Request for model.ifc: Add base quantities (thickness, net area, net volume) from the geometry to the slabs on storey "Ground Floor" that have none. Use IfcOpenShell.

First a look at what the model holds.

```python
import ifcopenshell
import ifcopenshell.util.element
import ifcopenshell.util.unit

model = ifcopenshell.open("model.ifc")
print(model.schema)
for unit_type in ("LENGTHUNIT", "AREAUNIT", "VOLUMEUNIT"):
    print(unit_type, ifcopenshell.util.unit.calculate_unit_scale(model, unit_type))
storey = next(s for s in model.by_type("IfcBuildingStorey") if s.Name == "Ground Floor")
slabs = [e for e in ifcopenshell.util.element.get_decomposition(storey) if e.is_a("IfcSlab")]
for e in sorted(slabs, key=lambda e: e.id()):
    print(e.id(), e.is_a(), e.Name, list(ifcopenshell.util.element.get_psets(e, qtos_only=True)), sep=" | ")
```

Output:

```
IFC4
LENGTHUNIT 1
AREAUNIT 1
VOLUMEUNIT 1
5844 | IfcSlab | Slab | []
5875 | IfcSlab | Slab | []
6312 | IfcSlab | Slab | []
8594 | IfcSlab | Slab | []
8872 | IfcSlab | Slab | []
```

```python
import ifcopenshell
import ifcopenshell.api.pset
import ifcopenshell.geom
import ifcopenshell.util.element
import ifcopenshell.util.shape
import ifcopenshell.util.unit

model = ifcopenshell.open("model.ifc")
unit_scale = ifcopenshell.util.unit.calculate_unit_scale(model)
area_scale = ifcopenshell.util.unit.calculate_unit_scale(model, "AREAUNIT")
volume_scale = ifcopenshell.util.unit.calculate_unit_scale(model, "VOLUMEUNIT")
settings = ifcopenshell.geom.settings()

storey = next(s for s in model.by_type("IfcBuildingStorey") if s.Name == "Ground Floor")
slabs = [e for e in ifcopenshell.util.element.get_decomposition(storey) if e.is_a("IfcSlab")]

for e in sorted(slabs, key=lambda e: e.id()):
    if ifcopenshell.util.element.get_psets(e, qtos_only=True, should_inherit=False):
        continue
    # Geometry comes back in metres, in the element's own axes.
    shape = ifcopenshell.geom.create_shape(settings, e)
    values = {
        "Width": ifcopenshell.util.shape.get_z(shape.geometry) / unit_scale,
        "NetArea": ifcopenshell.util.shape.get_footprint_area(shape.geometry) / area_scale,
        "NetVolume": ifcopenshell.util.shape.get_volume(shape.geometry) / volume_scale,
    }
    qto = ifcopenshell.api.pset.add_qto(model, product=e, name="Qto_SlabBaseQuantities")
    ifcopenshell.api.pset.edit_qto(model, qto=qto, properties=values)
    print(e.id(), {k: round(v, 3) for k, v in values.items()})

model.write("model_updated.ifc")
```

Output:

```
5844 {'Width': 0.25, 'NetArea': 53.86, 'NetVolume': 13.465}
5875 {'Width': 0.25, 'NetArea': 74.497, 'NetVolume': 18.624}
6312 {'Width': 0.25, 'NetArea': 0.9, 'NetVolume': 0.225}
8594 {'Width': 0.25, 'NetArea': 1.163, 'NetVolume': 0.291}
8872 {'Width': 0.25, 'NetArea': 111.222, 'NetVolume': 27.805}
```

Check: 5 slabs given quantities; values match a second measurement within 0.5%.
